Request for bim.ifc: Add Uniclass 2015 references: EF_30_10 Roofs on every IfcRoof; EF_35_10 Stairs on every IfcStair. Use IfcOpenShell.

First a look at what the model holds.

```python
import ifcopenshell

model = ifcopenshell.open("bim.ifc")
print(model.schema)
print("classifications:", [c.Name for c in model.by_type("IfcClassification")])
for ifc_class in ("IfcDoor", "IfcRoof", "IfcStair", "IfcWall", "IfcWindow"):
    print(ifc_class, len(model.by_type(ifc_class)))
```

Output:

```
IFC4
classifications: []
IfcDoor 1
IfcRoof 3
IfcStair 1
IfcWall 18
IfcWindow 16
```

```python
import ifcopenshell
import ifcopenshell.api.classification

model = ifcopenshell.open("bim.ifc")

system = ifcopenshell.api.classification.add_classification(model, classification="Uniclass 2015")

codes = {
    "IfcRoof": ("EF_30_10", "Roofs"),
    "IfcStair": ("EF_35_10", "Stairs"),
}
for ifc_class, (code, name) in codes.items():
    products = model.by_type(ifc_class)
    ifcopenshell.api.classification.add_reference(
        model, products=products, classification=system, identification=code, name=name
    )
    print(code, len(products))

model.write("bim_updated.ifc")
```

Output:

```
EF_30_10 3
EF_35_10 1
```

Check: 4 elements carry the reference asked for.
